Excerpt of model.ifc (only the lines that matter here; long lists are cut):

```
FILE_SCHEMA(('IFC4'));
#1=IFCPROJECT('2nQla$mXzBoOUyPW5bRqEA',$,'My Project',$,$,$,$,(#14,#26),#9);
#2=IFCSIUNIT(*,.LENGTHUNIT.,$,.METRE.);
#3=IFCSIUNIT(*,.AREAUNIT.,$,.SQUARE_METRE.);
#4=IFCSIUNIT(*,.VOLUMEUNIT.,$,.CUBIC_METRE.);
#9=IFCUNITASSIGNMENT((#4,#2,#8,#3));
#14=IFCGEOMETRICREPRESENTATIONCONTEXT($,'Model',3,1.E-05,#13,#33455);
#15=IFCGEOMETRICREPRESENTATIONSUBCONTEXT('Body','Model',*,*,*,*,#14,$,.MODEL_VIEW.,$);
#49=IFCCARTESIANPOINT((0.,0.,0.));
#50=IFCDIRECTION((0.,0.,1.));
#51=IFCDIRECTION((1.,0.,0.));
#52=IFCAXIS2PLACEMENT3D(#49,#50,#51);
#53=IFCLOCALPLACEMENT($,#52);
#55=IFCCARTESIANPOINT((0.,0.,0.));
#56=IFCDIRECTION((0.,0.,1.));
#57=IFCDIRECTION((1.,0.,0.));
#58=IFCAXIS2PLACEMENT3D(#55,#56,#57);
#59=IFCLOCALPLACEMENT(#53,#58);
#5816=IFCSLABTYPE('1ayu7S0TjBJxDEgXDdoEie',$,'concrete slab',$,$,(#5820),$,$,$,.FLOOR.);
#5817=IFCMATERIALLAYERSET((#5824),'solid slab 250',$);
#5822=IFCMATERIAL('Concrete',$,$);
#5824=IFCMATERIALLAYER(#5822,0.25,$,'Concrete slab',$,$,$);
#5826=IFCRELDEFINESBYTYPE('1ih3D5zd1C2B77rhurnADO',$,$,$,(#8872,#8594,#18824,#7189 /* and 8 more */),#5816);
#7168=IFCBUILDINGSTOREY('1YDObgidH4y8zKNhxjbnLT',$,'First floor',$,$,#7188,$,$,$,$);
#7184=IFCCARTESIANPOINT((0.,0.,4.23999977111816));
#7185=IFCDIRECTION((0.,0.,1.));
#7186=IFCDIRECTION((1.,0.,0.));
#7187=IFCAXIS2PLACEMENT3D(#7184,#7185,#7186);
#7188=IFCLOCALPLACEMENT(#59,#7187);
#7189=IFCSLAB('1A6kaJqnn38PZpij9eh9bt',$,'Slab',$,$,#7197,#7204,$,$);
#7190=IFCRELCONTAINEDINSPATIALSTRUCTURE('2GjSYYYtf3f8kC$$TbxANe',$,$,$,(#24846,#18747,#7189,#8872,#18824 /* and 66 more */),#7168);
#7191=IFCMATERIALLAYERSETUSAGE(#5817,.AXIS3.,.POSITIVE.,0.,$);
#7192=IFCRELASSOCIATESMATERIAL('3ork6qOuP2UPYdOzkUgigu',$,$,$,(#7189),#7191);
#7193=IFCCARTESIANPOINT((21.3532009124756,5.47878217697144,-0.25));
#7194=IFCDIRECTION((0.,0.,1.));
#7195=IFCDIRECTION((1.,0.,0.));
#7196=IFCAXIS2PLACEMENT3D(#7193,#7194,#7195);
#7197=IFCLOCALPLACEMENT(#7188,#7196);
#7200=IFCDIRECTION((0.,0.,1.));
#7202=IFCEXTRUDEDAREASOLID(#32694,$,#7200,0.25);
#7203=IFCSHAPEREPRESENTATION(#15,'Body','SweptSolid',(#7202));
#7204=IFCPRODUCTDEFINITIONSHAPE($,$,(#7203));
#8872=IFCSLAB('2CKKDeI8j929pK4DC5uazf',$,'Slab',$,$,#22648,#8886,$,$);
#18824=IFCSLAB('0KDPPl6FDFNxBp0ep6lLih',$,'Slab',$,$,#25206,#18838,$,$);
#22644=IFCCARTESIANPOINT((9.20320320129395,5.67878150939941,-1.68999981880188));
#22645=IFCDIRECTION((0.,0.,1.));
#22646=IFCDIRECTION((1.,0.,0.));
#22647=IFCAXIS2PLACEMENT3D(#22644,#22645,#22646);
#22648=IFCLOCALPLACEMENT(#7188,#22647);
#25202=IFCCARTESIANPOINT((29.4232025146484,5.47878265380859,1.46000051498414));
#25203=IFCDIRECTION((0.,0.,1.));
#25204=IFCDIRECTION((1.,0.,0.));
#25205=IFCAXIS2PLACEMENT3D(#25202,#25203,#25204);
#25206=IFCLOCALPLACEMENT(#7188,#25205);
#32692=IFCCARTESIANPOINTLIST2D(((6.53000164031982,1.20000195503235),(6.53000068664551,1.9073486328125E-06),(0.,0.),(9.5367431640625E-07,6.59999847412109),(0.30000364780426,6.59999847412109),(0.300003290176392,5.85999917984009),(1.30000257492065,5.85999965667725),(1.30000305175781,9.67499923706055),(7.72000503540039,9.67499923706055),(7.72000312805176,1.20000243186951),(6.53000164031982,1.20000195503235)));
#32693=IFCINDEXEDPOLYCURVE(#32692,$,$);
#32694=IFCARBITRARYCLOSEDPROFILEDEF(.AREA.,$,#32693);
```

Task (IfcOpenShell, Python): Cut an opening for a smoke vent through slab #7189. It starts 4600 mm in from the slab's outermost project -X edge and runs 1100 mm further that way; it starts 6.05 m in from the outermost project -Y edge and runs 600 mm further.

```python
import numpy as np
import ifcopenshell
import ifcopenshell.api.feature
import ifcopenshell.api.geometry
import ifcopenshell.api.root
import ifcopenshell.geom
import ifcopenshell.util.placement
import ifcopenshell.util.representation
import ifcopenshell.util.shape
import ifcopenshell.util.unit

model = ifcopenshell.open("model.ifc")
unit_scale = ifcopenshell.util.unit.calculate_unit_scale(model)
settings = ifcopenshell.geom.settings()


def volume(element):
    """Net volume in cubic metres, openings subtracted."""
    shape = ifcopenshell.geom.create_shape(settings, element)
    return ifcopenshell.util.shape.get_volume(shape.geometry)


slab = model.by_id(7189)
before = volume(slab)

# Extent in the slab's own axes, in metres. The edges named are its -X and -Y sides.
slab_shape = ifcopenshell.geom.create_shape(settings, slab)
vertices = ifcopenshell.util.shape.get_vertices(slab_shape.geometry)
x_min, y_min, bottom = vertices.min(axis=0)
top = vertices[:, 2].max()

opening = ifcopenshell.api.root.create_entity(model, ifc_class="IfcOpeningElement", name="Smoke vent opening", predefined_type="OPENING")
context = ifcopenshell.util.representation.get_context(model, "Model", "Body", "MODEL_VIEW")
width, depth = 1.1, 0.6
outline = [(0.0, 0.0), (width, 0.0), (width, depth), (0.0, depth), (0.0, 0.0)]
# Overshoot both faces by 50 mm so the cut is clean.
shape = ifcopenshell.api.geometry.add_slab_representation(
    model, context=context, depth=top - bottom + 0.1, polyline=outline
)
ifcopenshell.api.geometry.assign_representation(model, product=opening, representation=shape)

matrix = ifcopenshell.util.placement.get_local_placement(slab.ObjectPlacement)
matrix[:, 3] = matrix @ np.append(np.array([x_min + 4.6, y_min + 6.05, bottom - 0.05]) / unit_scale, 1.0)
ifcopenshell.api.geometry.edit_object_placement(model, product=opening, matrix=matrix, is_si=False)
ifcopenshell.api.feature.add_feature(model, feature=opening, element=slab)

after = volume(slab)

print(f"slab volume {before:.3f} -> {after:.3f} m3")

model.write("model-out.ifc")
```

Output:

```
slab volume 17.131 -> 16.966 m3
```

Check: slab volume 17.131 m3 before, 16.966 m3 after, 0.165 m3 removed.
